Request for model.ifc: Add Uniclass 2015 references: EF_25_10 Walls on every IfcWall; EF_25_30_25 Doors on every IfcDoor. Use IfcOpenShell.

First a look at what the model holds.

```python
import ifcopenshell

model = ifcopenshell.open("model.ifc")
print(model.schema)
print("classifications:", [c.Name for c in model.by_type("IfcClassification")])
for ifc_class in ("IfcDoor", "IfcRoof", "IfcStair", "IfcWall", "IfcWindow"):
    print(ifc_class, len(model.by_type(ifc_class)))
```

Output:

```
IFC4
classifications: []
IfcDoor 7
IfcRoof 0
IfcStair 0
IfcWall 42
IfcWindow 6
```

```python
import ifcopenshell
import ifcopenshell.api.classification

model = ifcopenshell.open("model.ifc")

system = ifcopenshell.api.classification.add_classification(model, classification="Uniclass 2015")

codes = {
    "IfcWall": ("EF_25_10", "Walls"),
    "IfcDoor": ("EF_25_30_25", "Doors"),
}
for ifc_class, (code, name) in codes.items():
    products = model.by_type(ifc_class)
    ifcopenshell.api.classification.add_reference(
        model, products=products, classification=system, identification=code, name=name
    )
    print(code, len(products))

model.write("model_v2.ifc")
```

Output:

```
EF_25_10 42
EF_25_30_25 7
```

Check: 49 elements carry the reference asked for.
